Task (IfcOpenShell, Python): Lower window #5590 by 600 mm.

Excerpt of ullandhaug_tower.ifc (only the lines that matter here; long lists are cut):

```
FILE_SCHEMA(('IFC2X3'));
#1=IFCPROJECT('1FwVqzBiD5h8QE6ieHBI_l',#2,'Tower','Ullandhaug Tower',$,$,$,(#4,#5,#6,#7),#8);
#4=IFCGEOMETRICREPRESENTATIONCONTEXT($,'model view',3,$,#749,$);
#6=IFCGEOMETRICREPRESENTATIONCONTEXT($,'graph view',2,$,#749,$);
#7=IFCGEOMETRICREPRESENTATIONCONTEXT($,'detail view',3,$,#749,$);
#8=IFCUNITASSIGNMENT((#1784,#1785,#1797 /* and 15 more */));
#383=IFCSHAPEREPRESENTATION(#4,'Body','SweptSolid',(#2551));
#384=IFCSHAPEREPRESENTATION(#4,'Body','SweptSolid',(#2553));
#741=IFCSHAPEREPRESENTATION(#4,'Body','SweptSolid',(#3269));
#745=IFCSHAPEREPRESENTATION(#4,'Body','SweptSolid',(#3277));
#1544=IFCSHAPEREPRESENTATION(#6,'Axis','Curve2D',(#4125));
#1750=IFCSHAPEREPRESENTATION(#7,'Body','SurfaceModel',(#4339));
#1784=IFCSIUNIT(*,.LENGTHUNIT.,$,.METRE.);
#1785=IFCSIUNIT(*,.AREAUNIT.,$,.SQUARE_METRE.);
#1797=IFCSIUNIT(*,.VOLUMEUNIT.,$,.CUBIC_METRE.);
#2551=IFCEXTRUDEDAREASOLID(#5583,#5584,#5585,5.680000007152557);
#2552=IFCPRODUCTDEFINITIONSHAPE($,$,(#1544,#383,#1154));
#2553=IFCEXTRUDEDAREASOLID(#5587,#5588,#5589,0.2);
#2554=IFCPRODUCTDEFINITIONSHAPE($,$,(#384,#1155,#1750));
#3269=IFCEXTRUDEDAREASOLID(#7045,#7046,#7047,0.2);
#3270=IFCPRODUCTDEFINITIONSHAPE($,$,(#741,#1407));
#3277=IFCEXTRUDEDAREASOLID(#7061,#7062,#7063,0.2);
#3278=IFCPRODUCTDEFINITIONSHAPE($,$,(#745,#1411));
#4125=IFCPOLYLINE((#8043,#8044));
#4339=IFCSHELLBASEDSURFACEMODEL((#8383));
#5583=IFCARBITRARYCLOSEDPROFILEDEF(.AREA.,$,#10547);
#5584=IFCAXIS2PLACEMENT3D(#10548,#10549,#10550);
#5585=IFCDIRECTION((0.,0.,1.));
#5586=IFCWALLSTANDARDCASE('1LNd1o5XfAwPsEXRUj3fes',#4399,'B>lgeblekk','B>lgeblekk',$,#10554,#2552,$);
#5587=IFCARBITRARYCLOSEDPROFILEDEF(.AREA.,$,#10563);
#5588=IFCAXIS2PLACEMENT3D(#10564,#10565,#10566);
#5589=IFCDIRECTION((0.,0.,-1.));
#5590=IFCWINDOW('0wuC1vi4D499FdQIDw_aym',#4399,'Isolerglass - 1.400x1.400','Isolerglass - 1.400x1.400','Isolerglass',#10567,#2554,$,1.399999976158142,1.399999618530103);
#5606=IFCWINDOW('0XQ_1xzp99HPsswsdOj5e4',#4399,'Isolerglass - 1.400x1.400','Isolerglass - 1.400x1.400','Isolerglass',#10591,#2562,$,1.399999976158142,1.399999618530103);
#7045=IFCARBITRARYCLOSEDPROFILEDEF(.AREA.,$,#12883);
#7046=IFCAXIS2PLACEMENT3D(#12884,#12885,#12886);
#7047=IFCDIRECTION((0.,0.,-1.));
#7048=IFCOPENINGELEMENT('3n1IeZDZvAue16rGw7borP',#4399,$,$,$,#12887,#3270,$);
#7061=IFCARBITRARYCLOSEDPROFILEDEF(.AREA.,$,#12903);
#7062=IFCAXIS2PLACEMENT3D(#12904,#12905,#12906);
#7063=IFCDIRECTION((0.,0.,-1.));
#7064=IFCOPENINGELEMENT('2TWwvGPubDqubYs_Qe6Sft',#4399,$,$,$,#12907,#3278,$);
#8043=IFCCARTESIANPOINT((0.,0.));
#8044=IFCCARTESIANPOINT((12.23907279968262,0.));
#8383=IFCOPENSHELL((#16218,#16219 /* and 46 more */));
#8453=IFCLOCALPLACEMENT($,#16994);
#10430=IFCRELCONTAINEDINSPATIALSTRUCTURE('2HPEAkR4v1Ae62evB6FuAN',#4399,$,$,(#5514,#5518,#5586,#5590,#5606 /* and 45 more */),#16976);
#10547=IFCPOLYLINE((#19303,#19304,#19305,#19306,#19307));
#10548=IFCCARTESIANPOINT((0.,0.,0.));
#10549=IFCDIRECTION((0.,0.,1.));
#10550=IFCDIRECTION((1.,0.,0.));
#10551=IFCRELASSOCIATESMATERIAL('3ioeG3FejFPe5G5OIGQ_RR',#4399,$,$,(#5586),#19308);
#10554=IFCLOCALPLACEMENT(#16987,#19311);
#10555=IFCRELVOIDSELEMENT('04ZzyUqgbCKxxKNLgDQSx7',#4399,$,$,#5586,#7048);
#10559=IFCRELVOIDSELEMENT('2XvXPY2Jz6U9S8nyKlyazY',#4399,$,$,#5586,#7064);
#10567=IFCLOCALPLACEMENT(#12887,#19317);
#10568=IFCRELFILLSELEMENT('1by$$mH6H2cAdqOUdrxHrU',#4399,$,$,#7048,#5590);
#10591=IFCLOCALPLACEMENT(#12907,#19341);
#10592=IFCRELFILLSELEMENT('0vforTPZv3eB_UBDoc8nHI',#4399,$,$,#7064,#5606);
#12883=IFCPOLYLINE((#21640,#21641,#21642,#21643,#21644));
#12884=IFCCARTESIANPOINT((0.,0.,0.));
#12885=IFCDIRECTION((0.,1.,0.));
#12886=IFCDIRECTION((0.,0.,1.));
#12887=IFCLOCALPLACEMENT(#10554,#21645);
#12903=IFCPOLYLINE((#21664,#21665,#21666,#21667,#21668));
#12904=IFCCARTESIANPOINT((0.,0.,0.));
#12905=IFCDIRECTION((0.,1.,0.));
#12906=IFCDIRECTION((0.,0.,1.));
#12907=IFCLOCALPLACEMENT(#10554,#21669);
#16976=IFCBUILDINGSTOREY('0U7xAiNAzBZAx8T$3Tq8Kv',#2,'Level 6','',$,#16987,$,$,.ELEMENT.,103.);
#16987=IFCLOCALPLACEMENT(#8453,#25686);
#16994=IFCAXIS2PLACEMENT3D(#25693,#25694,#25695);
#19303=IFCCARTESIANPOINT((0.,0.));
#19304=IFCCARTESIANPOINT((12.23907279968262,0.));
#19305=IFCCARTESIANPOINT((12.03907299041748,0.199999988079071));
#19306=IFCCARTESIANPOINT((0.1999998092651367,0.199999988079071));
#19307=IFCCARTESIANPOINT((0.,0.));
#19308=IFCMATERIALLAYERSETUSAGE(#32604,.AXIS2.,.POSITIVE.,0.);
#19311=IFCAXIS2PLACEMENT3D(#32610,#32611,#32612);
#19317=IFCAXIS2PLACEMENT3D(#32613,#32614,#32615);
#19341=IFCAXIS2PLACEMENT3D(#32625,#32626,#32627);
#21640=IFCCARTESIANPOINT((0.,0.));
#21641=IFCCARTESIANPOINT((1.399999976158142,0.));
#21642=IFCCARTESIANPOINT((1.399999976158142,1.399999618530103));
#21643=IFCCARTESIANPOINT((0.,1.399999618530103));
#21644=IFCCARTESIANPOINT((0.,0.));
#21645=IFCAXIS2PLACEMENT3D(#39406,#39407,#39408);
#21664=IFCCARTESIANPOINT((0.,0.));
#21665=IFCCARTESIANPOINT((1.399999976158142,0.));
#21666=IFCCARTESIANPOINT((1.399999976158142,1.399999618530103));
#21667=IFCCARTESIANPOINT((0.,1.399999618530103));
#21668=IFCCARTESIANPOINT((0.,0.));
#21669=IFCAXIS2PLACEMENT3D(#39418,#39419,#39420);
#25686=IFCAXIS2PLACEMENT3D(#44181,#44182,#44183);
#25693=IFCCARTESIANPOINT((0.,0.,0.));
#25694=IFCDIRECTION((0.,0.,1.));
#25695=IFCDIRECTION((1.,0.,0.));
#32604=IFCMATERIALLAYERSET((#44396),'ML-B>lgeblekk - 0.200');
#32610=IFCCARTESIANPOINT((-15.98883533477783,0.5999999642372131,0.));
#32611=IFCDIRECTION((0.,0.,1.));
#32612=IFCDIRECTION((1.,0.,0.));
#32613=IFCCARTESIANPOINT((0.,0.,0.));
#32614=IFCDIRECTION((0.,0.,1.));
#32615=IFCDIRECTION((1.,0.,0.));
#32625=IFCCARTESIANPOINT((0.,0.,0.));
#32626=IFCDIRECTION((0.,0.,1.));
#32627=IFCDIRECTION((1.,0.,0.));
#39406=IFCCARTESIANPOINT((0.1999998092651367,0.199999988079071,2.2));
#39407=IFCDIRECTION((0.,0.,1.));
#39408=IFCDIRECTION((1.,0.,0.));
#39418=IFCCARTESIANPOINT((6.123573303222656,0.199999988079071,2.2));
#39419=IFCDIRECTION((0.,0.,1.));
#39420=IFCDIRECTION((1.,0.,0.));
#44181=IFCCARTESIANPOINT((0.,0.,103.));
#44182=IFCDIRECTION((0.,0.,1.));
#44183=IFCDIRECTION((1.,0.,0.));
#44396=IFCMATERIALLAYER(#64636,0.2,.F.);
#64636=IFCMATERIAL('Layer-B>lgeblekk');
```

```python
import numpy as np
import ifcopenshell
import ifcopenshell.api.geometry
import ifcopenshell.util.placement
import ifcopenshell.util.unit

model = ifcopenshell.open("ullandhaug_tower.ifc")
unit_scale = ifcopenshell.util.unit.calculate_unit_scale(model)

window = model.by_id(5590)
opening = window.FillsVoids[0].RelatingOpeningElement
dz = -0.6 / unit_scale

shift = np.array([0.0, 0.0, dz])
# The window is placed relative to its opening, so it follows when the opening moves.
matrix = ifcopenshell.util.placement.get_local_placement(opening.ObjectPlacement)
matrix[:3, 3] += shift
ifcopenshell.api.geometry.edit_object_placement(
    model, product=opening, matrix=matrix, is_si=False, should_transform_children=True
)

print(f"moved by {dz * unit_scale:+.3f} m")

model.write("ullandhaug_tower_v2.ifc")
```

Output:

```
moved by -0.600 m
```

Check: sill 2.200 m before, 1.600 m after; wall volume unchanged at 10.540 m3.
